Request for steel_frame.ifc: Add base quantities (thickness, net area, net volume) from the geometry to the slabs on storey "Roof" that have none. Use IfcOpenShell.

First a look at what the model holds.

```python
import ifcopenshell
import ifcopenshell.util.element
import ifcopenshell.util.unit

model = ifcopenshell.open("steel_frame.ifc")
print(model.schema)
for unit_type in ("LENGTHUNIT", "AREAUNIT", "VOLUMEUNIT"):
    print(unit_type, ifcopenshell.util.unit.calculate_unit_scale(model, unit_type))
storey = next(s for s in model.by_type("IfcBuildingStorey") if s.Name == "Roof")
slabs = [e for e in ifcopenshell.util.element.get_decomposition(storey) if e.is_a("IfcSlab")]
for e in sorted(slabs, key=lambda e: e.id()):
    print(e.id(), e.is_a(), e.Name, list(ifcopenshell.util.element.get_psets(e, qtos_only=True)), sep=" | ")
```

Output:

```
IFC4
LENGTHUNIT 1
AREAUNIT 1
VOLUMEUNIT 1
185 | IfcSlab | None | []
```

```python
import ifcopenshell
import ifcopenshell.api.pset
import ifcopenshell.geom
import ifcopenshell.util.element
import ifcopenshell.util.shape
import ifcopenshell.util.unit

model = ifcopenshell.open("steel_frame.ifc")
unit_scale = ifcopenshell.util.unit.calculate_unit_scale(model)
area_scale = ifcopenshell.util.unit.calculate_unit_scale(model, "AREAUNIT")
volume_scale = ifcopenshell.util.unit.calculate_unit_scale(model, "VOLUMEUNIT")
settings = ifcopenshell.geom.settings()

storey = next(s for s in model.by_type("IfcBuildingStorey") if s.Name == "Roof")
slabs = [e for e in ifcopenshell.util.element.get_decomposition(storey) if e.is_a("IfcSlab")]

for e in sorted(slabs, key=lambda e: e.id()):
    if ifcopenshell.util.element.get_psets(e, qtos_only=True, should_inherit=False):
        continue
    # Geometry comes back in metres, in the element's own axes.
    shape = ifcopenshell.geom.create_shape(settings, e)
    values = {
        "Width": ifcopenshell.util.shape.get_z(shape.geometry) / unit_scale,
        "NetArea": ifcopenshell.util.shape.get_footprint_area(shape.geometry) / area_scale,
        "NetVolume": ifcopenshell.util.shape.get_volume(shape.geometry) / volume_scale,
    }
    qto = ifcopenshell.api.pset.add_qto(model, product=e, name="Qto_SlabBaseQuantities")
    ifcopenshell.api.pset.edit_qto(model, qto=qto, properties=values)
    print(e.id(), {k: round(v, 3) for k, v in values.items()})

model.write("steel_frame_updated.ifc")
```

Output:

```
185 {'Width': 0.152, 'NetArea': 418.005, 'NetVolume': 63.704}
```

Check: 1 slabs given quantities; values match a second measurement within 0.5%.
